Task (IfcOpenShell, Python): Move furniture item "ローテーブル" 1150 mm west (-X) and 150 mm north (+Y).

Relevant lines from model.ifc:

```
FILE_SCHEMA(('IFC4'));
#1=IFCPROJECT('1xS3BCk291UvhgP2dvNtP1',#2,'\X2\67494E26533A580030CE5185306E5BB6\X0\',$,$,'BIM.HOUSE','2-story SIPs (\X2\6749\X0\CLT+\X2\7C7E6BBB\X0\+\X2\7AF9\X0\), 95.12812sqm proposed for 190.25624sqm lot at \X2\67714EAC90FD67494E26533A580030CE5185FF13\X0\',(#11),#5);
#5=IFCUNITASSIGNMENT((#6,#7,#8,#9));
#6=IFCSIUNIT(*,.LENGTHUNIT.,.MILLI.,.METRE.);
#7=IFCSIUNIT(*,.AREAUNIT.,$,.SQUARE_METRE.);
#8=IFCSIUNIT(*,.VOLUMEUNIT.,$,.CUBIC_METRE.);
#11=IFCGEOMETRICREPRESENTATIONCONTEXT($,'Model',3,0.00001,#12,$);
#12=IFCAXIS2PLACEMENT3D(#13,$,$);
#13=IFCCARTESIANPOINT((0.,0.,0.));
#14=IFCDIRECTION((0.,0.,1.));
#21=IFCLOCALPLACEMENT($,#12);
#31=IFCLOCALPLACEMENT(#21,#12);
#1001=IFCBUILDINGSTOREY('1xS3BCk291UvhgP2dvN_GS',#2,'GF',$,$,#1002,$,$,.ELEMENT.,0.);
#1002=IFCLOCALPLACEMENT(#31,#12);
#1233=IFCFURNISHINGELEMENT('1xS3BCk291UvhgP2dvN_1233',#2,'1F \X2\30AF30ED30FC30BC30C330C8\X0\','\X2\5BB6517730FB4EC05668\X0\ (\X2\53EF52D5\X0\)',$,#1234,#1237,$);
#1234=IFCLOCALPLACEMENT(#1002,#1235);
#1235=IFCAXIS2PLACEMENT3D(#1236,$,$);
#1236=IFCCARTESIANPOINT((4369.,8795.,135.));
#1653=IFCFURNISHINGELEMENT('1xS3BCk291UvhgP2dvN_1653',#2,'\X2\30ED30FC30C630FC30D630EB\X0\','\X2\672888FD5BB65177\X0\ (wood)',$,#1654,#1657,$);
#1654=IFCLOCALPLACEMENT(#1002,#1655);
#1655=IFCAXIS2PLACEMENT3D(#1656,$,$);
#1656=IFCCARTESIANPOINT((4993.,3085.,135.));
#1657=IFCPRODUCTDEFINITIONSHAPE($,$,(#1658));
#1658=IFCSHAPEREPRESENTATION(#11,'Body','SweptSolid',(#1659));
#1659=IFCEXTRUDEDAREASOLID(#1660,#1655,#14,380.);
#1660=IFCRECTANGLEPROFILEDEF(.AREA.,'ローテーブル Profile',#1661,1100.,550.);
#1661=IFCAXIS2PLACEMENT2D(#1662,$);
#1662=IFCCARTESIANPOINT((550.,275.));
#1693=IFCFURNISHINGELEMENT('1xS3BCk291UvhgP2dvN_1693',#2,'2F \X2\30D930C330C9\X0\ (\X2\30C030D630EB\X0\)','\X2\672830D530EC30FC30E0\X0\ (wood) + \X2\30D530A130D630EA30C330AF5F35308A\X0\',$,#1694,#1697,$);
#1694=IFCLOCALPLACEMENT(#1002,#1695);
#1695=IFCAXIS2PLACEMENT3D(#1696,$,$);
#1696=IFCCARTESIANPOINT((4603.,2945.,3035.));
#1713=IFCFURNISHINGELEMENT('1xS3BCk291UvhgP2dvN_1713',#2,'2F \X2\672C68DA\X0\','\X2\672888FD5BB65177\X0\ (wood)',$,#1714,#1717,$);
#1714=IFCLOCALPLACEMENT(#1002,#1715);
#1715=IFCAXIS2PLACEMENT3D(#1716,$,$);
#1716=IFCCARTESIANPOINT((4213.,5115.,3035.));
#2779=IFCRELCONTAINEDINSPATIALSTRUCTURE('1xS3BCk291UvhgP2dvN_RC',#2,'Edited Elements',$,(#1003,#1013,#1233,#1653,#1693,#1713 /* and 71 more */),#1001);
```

```python
import ifcopenshell
import ifcopenshell.api.geometry
import ifcopenshell.util.placement
import ifcopenshell.util.unit

model = ifcopenshell.open("model.ifc")
unit_scale = ifcopenshell.util.unit.calculate_unit_scale(model)

item = model.by_guid("1xS3BCk291UvhgP2dvN_1653")
matrix = ifcopenshell.util.placement.get_local_placement(item.ObjectPlacement)
matrix[0, 3] -= 1.15 / unit_scale
matrix[1, 3] += 0.15 / unit_scale
ifcopenshell.api.geometry.edit_object_placement(model, product=item, matrix=matrix, is_si=False)

print(ifcopenshell.util.placement.get_local_placement(item.ObjectPlacement).round(3) + 0.0)

model.write("model_rev.ifc")
```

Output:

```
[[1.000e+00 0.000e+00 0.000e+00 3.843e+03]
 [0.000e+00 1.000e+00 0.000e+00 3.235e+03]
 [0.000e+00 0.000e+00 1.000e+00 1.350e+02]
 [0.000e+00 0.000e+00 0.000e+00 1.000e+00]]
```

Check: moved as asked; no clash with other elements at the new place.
